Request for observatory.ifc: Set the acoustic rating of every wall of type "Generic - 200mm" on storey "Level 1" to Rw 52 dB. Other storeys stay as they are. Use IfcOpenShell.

First a look at what the model holds.

```python
import ifcopenshell
import ifcopenshell.util.element

model = ifcopenshell.open("observatory.ifc")
print(model.schema)
storey = next(s for s in model.by_type("IfcBuildingStorey") if s.Name == "Level 1")
walls = [e for e in ifcopenshell.util.element.get_decomposition(storey) if e.is_a("IfcWall")]
seen = {}
for e in walls:
    element_type = ifcopenshell.util.element.get_type(e)
    key = (element_type.Name if element_type != e and element_type else None, ifcopenshell.util.element.get_pset(e, "Pset_WallCommon", "AcousticRating"))
    seen[key] = seen.get(key, 0) + 1
for (name, value), count in sorted(seen.items(), key=str):
    print(count, "x", name, "|", value)
```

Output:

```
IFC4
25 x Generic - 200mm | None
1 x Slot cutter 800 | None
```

```python
import ifcopenshell
import ifcopenshell.api.pset
import ifcopenshell.util.element

model = ifcopenshell.open("observatory.ifc")

storey = next(s for s in model.by_type("IfcBuildingStorey") if s.Name == "Level 1")
walls = [e for e in ifcopenshell.util.element.get_decomposition(storey) if e.is_a("IfcWall")]

count = 0
for e in walls:
    element_type = ifcopenshell.util.element.get_type(e)
    if element_type in (None, e) or element_type.Name != "Generic - 200mm":
        continue
    # add_pset returns the element's existing set when there is one.
    pset = ifcopenshell.api.pset.add_pset(model, product=e, name="Pset_WallCommon")
    ifcopenshell.api.pset.edit_pset(model, pset=pset, properties={"AcousticRating": "Rw 52 dB"})
    count += 1

print(count, "walls updated")

model.write("observatory_updated.ifc")
```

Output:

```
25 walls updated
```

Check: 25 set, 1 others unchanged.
